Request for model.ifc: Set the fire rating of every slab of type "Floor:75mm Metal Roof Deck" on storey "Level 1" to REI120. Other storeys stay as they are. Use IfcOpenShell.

First a look at what the model holds.

```python
import ifcopenshell
import ifcopenshell.util.element

model = ifcopenshell.open("model.ifc")
print(model.schema)
storey = next(s for s in model.by_type("IfcBuildingStorey") if s.Name == "Level 1")
slabs = [e for e in ifcopenshell.util.element.get_decomposition(storey) if e.is_a("IfcSlab")]
seen = {}
for e in slabs:
    element_type = ifcopenshell.util.element.get_type(e)
    key = (element_type.Name if element_type != e and element_type else None, ifcopenshell.util.element.get_pset(e, "Pset_SlabCommon", "FireRating"))
    seen[key] = seen.get(key, 0) + 1
for (name, value), count in sorted(seen.items(), key=str):
    print(count, "x", name, "|", value)
```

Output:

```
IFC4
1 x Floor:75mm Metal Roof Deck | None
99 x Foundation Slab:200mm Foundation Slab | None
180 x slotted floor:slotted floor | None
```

```python
import ifcopenshell
import ifcopenshell.api.pset
import ifcopenshell.util.element

model = ifcopenshell.open("model.ifc")

storey = next(s for s in model.by_type("IfcBuildingStorey") if s.Name == "Level 1")
slabs = [e for e in ifcopenshell.util.element.get_decomposition(storey) if e.is_a("IfcSlab")]

count = 0
for e in slabs:
    element_type = ifcopenshell.util.element.get_type(e)
    if element_type in (None, e) or element_type.Name != "Floor:75mm Metal Roof Deck":
        continue
    # add_pset returns the element's existing set when there is one.
    pset = ifcopenshell.api.pset.add_pset(model, product=e, name="Pset_SlabCommon")
    ifcopenshell.api.pset.edit_pset(model, pset=pset, properties={"FireRating": "REI120"})
    count += 1

print(count, "slabs updated")

model.write("model-out.ifc")
```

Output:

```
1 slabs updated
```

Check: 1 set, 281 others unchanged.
